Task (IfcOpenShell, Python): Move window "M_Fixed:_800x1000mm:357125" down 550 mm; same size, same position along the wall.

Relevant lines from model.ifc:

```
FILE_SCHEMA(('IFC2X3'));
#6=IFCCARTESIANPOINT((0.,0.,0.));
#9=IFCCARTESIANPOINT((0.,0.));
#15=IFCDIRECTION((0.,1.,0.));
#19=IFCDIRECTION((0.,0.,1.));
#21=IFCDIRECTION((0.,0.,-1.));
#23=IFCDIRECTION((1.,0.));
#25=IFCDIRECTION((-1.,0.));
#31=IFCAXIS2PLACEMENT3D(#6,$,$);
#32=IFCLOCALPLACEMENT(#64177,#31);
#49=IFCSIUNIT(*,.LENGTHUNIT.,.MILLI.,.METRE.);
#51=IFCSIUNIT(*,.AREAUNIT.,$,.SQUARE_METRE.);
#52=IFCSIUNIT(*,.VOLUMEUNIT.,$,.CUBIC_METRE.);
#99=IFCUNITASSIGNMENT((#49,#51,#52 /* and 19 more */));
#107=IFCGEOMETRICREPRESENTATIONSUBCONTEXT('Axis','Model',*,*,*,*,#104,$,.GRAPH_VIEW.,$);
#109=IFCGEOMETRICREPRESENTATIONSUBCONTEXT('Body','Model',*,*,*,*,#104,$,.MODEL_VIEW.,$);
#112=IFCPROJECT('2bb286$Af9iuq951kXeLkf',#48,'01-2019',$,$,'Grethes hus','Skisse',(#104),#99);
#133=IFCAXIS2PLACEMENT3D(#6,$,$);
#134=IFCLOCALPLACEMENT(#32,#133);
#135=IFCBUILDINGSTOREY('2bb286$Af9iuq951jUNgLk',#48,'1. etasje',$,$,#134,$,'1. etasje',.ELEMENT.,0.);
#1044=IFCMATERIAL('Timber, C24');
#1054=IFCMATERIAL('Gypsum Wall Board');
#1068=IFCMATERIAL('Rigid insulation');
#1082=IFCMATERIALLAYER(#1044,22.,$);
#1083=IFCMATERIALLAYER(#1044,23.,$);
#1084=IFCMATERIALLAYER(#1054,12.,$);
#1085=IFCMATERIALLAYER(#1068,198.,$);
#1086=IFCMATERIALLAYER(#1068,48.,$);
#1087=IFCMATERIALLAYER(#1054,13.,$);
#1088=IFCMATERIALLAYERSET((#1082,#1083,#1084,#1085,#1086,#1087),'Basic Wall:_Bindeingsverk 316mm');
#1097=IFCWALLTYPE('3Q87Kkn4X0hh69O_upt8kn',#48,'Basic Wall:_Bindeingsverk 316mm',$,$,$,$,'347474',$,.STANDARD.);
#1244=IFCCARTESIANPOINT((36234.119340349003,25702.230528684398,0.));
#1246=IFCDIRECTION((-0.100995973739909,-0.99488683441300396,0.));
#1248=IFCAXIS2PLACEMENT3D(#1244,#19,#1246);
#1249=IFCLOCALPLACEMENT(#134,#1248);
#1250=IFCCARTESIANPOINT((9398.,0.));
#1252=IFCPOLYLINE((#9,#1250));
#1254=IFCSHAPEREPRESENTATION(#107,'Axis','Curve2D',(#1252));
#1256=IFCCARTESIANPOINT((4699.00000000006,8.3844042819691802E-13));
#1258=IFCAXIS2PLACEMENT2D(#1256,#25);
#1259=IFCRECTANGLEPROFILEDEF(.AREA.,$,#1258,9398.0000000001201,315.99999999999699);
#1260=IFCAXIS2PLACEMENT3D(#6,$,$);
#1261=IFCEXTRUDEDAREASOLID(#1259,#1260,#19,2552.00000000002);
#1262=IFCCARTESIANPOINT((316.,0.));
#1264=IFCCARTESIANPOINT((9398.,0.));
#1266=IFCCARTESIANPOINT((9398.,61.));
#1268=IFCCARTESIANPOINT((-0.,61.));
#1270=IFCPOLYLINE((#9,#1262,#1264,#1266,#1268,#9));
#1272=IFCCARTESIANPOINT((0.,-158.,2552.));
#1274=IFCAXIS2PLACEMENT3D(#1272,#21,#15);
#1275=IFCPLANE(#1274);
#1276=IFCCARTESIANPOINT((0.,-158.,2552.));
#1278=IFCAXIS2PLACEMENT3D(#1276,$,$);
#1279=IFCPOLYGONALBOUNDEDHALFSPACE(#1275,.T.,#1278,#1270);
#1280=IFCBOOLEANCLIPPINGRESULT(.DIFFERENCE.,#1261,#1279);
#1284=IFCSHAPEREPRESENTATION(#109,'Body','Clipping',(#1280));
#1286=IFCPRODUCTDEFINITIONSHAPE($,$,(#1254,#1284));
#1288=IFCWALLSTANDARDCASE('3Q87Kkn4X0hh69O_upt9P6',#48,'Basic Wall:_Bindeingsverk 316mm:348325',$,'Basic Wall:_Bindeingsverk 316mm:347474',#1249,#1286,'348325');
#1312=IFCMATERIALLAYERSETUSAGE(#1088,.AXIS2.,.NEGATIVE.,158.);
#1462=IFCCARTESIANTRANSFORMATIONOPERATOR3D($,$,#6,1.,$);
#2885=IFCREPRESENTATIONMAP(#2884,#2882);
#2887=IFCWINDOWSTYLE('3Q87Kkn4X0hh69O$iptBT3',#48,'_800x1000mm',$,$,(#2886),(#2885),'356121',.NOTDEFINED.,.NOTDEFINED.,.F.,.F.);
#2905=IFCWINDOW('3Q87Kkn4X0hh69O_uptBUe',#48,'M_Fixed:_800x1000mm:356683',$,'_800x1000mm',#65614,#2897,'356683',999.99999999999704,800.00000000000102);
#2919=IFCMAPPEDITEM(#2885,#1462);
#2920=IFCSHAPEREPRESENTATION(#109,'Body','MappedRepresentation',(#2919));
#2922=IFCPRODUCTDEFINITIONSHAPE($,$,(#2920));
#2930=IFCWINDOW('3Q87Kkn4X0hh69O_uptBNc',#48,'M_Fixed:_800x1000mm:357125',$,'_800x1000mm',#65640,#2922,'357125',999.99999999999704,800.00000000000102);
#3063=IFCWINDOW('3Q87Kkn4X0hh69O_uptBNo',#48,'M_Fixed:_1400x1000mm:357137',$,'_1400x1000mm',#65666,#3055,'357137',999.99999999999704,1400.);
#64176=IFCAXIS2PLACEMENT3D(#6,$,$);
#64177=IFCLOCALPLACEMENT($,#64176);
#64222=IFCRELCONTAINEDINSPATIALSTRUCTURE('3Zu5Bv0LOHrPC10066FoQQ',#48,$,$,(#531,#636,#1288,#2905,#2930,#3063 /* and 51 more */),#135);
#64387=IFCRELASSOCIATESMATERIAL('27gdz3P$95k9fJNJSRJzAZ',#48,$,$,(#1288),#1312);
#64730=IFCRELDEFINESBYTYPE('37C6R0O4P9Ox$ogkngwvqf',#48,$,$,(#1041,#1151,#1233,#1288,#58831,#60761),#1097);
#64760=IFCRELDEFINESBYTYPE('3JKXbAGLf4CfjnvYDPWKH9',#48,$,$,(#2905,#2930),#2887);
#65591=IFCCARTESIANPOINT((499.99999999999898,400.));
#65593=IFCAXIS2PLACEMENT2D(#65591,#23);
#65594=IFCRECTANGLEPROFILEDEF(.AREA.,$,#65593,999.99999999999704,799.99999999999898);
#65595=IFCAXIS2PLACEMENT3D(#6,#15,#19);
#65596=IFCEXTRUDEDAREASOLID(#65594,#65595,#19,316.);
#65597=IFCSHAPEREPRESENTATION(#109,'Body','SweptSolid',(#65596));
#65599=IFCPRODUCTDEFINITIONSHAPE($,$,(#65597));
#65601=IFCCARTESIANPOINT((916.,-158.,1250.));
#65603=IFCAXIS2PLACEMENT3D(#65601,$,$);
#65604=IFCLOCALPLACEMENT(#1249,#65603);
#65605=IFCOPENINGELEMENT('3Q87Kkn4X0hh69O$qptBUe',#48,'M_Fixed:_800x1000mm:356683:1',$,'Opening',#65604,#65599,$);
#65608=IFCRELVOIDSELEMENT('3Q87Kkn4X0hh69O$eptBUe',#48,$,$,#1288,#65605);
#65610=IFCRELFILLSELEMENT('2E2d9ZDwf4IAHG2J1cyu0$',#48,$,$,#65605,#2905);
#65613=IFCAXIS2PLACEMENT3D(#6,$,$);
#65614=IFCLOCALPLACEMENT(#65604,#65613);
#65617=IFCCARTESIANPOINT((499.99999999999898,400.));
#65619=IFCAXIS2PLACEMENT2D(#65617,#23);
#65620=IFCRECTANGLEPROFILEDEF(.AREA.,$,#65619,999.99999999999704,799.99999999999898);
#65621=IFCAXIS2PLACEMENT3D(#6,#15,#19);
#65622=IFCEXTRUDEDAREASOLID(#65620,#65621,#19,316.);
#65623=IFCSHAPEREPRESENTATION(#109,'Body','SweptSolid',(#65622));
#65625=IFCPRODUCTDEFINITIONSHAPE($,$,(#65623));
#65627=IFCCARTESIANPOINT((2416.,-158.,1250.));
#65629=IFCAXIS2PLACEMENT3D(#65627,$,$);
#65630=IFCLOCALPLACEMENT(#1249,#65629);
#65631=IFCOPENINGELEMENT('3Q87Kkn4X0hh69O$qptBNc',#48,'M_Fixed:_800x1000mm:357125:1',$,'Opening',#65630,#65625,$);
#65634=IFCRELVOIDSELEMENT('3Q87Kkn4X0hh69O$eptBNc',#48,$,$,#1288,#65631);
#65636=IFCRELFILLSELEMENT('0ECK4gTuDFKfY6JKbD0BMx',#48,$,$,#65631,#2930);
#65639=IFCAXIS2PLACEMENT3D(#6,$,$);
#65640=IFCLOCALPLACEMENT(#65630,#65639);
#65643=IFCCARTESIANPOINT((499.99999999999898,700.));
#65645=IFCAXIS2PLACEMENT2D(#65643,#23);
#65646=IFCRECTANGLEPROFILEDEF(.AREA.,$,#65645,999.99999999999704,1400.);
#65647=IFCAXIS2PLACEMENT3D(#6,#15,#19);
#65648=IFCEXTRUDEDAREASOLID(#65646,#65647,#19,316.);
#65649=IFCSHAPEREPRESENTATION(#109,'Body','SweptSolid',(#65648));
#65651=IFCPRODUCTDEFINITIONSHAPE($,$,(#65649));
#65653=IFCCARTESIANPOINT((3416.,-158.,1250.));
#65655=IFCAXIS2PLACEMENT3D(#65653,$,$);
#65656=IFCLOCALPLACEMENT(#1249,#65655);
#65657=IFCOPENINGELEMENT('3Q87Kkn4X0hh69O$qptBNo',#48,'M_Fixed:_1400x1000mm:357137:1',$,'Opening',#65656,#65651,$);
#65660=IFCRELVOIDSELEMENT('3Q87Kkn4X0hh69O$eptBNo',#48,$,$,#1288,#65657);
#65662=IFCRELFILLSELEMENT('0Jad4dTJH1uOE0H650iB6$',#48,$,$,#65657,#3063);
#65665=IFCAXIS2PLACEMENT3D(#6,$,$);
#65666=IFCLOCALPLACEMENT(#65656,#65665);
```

```python
import numpy as np
import ifcopenshell
import ifcopenshell.api.geometry
import ifcopenshell.util.placement
import ifcopenshell.util.unit

model = ifcopenshell.open("model.ifc")
unit_scale = ifcopenshell.util.unit.calculate_unit_scale(model)

window = model.by_guid("3Q87Kkn4X0hh69O_uptBNc")
opening = window.FillsVoids[0].RelatingOpeningElement
dz = -550.0

shift = np.array([0.0, 0.0, dz])
# The window is placed relative to its opening, so it follows when the opening moves.
matrix = ifcopenshell.util.placement.get_local_placement(opening.ObjectPlacement)
matrix[:3, 3] += shift
ifcopenshell.api.geometry.edit_object_placement(
    model, product=opening, matrix=matrix, is_si=False, should_transform_children=True
)

print(f"moved by {dz * unit_scale:+.3f} m")

model.write("model-out.ifc")
```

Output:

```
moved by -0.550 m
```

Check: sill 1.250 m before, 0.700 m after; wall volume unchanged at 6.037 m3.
